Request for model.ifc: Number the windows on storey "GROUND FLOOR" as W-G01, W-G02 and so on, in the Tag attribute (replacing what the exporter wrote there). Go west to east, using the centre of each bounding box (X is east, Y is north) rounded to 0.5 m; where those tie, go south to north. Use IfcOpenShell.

First a look at what the model holds.

```python
import ifcopenshell
import ifcopenshell.util.element
import ifcopenshell.util.placement

model = ifcopenshell.open("model.ifc")
print(model.schema)
storey = next(s for s in model.by_type("IfcBuildingStorey") if s.Name == "GROUND FLOOR")
windows = [e for e in ifcopenshell.util.element.get_decomposition(storey) if e.is_a("IfcWindow")]
for e in sorted(windows, key=lambda e: e.id()):
    origin = ifcopenshell.util.placement.get_local_placement(e.ObjectPlacement)[:3, 3]
    print(e.id(), e.Tag, e.Name, origin.round(2) + 0.0, sep=" | ")
```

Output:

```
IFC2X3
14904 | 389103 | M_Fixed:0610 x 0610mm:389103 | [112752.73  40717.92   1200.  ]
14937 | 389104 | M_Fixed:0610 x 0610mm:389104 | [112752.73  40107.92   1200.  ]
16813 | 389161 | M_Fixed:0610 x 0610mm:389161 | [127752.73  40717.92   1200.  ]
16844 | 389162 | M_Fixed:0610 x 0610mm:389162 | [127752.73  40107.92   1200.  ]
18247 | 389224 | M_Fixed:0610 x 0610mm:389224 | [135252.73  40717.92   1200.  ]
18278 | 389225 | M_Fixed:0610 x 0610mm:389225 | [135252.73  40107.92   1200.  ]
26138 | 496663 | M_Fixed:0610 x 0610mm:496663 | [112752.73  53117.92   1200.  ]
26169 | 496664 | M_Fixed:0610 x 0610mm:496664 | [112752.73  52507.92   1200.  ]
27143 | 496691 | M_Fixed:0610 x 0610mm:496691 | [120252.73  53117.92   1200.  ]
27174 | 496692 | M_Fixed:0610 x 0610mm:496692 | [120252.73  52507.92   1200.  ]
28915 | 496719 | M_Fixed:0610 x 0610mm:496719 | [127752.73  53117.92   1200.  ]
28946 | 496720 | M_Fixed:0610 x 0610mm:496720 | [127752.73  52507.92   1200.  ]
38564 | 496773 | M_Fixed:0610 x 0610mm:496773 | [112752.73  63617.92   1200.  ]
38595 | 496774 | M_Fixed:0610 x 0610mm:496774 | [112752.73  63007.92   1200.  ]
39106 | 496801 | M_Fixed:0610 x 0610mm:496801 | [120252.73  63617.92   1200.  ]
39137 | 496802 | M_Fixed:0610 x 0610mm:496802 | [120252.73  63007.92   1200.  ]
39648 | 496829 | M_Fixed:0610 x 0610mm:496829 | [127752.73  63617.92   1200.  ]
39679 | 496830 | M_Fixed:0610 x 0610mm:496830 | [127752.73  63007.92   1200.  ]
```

```python
import ifcopenshell
import ifcopenshell.geom
import ifcopenshell.util.element
import ifcopenshell.util.shape

model = ifcopenshell.open("model.ifc")
settings = ifcopenshell.geom.settings()
settings.set("use-world-coords", True)


def centre(element):
    shape = ifcopenshell.geom.create_shape(settings, element)
    return ifcopenshell.util.shape.get_bbox_centroid(shape.geometry)


storey = next(s for s in model.by_type("IfcBuildingStorey") if s.Name == "GROUND FLOOR")
windows = [e for e in ifcopenshell.util.element.get_decomposition(storey) if e.is_a("IfcWindow")]

# Insertion points can sit at a corner or the storey origin, so sort by the geometry (in metres).
centres = {e: centre(e) for e in windows}
windows.sort(key=lambda e: (round(centres[e][0] / 0.5), centres[e][1]))

for i, e in enumerate(windows, start=1):
    number = f"W-G{i:02d}"
    e.Tag = number
    print(e.id(), number)

model.write("model-out.ifc")
```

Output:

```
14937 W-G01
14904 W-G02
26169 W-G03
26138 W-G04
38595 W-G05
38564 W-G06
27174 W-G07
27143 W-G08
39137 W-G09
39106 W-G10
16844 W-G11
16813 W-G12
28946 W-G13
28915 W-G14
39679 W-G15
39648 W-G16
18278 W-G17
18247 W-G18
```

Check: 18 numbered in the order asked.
